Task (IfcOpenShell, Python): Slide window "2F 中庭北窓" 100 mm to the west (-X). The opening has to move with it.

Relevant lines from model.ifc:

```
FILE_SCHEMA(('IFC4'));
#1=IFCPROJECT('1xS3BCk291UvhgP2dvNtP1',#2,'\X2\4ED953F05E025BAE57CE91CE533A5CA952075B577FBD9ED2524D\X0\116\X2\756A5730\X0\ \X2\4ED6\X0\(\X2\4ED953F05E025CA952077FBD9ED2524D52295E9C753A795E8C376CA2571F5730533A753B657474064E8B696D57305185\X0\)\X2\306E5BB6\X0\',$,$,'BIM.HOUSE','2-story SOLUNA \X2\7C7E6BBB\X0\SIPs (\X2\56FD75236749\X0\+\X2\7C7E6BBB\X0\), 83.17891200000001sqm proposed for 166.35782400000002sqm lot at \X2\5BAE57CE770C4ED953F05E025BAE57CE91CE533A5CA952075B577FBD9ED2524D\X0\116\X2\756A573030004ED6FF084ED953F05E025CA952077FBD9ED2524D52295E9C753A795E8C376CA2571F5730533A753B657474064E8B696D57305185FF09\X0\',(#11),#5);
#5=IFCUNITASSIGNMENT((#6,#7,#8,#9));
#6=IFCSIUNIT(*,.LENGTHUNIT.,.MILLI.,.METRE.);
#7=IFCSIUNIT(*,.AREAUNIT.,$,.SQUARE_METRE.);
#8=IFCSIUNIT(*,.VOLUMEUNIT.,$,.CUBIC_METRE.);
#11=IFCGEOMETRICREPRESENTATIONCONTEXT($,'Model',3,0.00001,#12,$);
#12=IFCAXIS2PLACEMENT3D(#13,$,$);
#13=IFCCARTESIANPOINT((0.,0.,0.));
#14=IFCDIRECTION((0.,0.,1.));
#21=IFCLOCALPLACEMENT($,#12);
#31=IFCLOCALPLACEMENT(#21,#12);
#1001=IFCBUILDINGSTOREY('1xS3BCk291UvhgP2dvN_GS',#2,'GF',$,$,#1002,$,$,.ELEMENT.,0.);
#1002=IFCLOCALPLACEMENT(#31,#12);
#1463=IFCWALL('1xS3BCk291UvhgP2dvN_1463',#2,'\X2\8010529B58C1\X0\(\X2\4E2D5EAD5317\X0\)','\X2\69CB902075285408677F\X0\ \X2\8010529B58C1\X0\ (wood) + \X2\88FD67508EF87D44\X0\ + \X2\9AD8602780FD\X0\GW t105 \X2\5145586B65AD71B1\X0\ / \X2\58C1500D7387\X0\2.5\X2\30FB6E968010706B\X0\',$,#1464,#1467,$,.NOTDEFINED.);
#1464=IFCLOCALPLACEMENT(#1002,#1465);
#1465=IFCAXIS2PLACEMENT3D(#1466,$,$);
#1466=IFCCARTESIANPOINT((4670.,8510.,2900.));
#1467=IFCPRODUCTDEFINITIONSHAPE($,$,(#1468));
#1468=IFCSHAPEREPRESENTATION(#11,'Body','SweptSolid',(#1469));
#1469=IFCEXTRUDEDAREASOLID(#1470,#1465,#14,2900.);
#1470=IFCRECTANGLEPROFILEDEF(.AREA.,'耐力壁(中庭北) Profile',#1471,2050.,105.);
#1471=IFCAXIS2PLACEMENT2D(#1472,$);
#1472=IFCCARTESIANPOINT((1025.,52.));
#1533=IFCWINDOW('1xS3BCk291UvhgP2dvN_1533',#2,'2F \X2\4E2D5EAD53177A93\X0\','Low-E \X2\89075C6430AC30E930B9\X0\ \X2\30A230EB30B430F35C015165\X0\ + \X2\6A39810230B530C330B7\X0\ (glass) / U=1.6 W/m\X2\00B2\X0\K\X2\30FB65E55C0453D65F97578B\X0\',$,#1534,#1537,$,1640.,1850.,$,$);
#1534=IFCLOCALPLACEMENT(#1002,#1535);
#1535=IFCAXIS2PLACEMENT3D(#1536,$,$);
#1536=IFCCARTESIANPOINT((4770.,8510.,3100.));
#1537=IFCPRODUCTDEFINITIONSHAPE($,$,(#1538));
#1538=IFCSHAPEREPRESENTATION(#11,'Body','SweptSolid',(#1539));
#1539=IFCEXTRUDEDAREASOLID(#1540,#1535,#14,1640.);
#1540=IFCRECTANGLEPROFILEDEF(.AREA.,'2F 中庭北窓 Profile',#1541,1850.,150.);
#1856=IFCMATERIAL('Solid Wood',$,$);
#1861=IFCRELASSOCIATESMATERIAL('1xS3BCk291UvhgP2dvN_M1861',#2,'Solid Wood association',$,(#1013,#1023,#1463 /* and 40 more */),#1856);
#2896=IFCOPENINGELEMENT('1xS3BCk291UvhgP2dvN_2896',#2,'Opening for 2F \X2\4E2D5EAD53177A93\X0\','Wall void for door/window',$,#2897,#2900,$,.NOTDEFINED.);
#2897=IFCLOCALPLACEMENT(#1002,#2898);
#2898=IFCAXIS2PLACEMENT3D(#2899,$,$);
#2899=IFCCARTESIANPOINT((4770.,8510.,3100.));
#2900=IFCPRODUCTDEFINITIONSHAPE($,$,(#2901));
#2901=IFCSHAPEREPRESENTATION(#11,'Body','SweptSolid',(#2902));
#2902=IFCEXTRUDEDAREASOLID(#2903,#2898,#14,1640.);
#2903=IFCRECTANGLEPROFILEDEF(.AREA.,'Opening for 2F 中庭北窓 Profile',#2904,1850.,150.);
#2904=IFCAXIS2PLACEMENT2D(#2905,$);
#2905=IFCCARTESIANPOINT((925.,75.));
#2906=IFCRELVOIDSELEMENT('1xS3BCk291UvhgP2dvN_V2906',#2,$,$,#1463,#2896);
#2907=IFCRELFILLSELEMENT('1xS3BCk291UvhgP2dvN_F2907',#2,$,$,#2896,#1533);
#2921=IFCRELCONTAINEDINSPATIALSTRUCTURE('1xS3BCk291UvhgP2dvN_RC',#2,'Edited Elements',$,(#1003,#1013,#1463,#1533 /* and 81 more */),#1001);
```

```python
import ifcopenshell
import ifcopenshell.api.geometry
import ifcopenshell.util.placement
import ifcopenshell.util.unit

model = ifcopenshell.open("model.ifc")
unit_scale = ifcopenshell.util.unit.calculate_unit_scale(model)

window = model.by_guid("1xS3BCk291UvhgP2dvN_1533")
opening = window.FillsVoids[0].RelatingOpeningElement
wall = opening.VoidsElements[0].RelatingBuildingElement

wall_matrix = ifcopenshell.util.placement.get_local_placement(wall.ObjectPlacement)
shift = wall_matrix[:3, 0] * -0.1 / unit_scale
before = ifcopenshell.util.placement.get_local_placement(window.ObjectPlacement)[:3, 3].copy()

# The window is not placed relative to its opening, so move both.
for product in (opening, window):
    matrix = ifcopenshell.util.placement.get_local_placement(product.ObjectPlacement)
    matrix[:3, 3] += shift
    ifcopenshell.api.geometry.edit_object_placement(model, product=product, matrix=matrix, is_si=False)

after = ifcopenshell.util.placement.get_local_placement(window.ObjectPlacement)[:3, 3]
print("window moved by", (after - before).round(3) + 0.0)

model.write("model_rev.ifc")
```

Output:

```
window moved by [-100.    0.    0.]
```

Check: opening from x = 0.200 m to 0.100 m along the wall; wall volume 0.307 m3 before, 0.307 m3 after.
